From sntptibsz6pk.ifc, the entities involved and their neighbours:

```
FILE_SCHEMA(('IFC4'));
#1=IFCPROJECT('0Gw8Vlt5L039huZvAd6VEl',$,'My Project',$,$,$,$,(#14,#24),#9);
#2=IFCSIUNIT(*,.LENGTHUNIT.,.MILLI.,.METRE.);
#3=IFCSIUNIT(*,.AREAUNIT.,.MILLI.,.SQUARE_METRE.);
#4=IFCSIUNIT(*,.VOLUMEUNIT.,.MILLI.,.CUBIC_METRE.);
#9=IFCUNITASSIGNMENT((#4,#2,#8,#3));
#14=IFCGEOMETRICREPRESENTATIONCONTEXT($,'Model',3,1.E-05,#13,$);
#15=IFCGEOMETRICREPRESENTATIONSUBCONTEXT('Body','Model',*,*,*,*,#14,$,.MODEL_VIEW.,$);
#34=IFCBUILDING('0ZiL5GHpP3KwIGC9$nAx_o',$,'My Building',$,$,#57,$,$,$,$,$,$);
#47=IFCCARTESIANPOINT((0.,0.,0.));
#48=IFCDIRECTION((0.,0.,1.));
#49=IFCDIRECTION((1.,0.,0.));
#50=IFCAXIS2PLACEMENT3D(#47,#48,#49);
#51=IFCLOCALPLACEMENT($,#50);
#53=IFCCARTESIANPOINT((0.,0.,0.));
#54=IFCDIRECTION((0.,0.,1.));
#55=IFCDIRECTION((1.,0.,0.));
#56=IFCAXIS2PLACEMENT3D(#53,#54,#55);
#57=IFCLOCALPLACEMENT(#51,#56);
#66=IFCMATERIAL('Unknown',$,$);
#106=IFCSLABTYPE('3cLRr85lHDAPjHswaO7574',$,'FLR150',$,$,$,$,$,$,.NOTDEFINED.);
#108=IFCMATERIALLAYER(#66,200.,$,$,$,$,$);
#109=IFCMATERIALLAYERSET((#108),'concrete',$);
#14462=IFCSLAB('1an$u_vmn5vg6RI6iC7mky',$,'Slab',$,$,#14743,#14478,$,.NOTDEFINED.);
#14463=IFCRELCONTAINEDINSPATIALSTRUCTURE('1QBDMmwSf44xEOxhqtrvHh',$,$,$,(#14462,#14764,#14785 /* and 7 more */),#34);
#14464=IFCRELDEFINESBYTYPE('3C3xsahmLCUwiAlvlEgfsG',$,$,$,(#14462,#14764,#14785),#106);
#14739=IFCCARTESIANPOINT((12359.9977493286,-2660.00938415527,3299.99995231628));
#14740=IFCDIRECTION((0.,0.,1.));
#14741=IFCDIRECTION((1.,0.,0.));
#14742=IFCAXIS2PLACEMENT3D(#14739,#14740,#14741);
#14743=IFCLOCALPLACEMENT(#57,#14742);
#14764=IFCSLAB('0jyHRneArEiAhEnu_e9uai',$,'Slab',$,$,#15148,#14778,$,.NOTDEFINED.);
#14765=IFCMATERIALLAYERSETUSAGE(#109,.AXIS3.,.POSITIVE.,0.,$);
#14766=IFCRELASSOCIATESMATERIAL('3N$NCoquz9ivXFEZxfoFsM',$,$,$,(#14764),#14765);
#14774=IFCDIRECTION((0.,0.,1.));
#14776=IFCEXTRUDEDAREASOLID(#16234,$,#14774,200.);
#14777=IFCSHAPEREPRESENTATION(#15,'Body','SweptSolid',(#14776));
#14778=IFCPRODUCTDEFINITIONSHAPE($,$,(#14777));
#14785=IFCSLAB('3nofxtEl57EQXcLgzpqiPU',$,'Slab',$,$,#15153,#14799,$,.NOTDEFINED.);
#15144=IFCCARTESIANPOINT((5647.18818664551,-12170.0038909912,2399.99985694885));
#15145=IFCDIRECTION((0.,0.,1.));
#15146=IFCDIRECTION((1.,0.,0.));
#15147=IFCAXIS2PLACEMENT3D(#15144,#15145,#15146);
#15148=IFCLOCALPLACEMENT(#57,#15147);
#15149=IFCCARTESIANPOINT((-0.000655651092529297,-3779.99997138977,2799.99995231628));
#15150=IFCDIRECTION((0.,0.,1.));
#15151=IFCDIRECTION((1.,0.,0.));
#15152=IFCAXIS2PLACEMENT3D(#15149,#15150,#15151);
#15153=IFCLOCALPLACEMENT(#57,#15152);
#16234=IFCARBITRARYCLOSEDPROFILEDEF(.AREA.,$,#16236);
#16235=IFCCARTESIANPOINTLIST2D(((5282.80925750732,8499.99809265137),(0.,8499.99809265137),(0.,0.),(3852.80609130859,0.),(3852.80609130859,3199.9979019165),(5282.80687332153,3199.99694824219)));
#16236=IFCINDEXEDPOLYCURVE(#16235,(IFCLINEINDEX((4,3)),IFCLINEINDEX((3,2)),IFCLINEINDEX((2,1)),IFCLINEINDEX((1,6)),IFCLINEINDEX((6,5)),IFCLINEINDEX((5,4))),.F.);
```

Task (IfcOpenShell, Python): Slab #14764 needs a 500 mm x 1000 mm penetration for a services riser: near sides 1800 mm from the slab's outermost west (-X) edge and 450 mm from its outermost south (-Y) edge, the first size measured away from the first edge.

```python
import numpy as np
import ifcopenshell
import ifcopenshell.api.feature
import ifcopenshell.api.geometry
import ifcopenshell.api.root
import ifcopenshell.geom
import ifcopenshell.util.placement
import ifcopenshell.util.representation
import ifcopenshell.util.shape
import ifcopenshell.util.unit

model = ifcopenshell.open("sntptibsz6pk.ifc")
unit_scale = ifcopenshell.util.unit.calculate_unit_scale(model)
settings = ifcopenshell.geom.settings()


def volume(element):
    """Net volume in cubic metres, openings subtracted."""
    shape = ifcopenshell.geom.create_shape(settings, element)
    return ifcopenshell.util.shape.get_volume(shape.geometry)


slab = model.by_guid("0jyHRneArEiAhEnu_e9uai")
before = volume(slab)

# Extent in the slab's own axes, in metres. The edges named are its -X and -Y sides.
slab_shape = ifcopenshell.geom.create_shape(settings, slab)
vertices = ifcopenshell.util.shape.get_vertices(slab_shape.geometry)
x_min, y_min, bottom = vertices.min(axis=0)
top = vertices[:, 2].max()

opening = ifcopenshell.api.root.create_entity(model, ifc_class="IfcOpeningElement", name="Services riser opening", predefined_type="OPENING")
context = ifcopenshell.util.representation.get_context(model, "Model", "Body", "MODEL_VIEW")
width, depth = 0.5, 1
outline = [(0.0, 0.0), (width, 0.0), (width, depth), (0.0, depth), (0.0, 0.0)]
# Overshoot both faces by 50 mm so the cut is clean.
shape = ifcopenshell.api.geometry.add_slab_representation(
    model, context=context, depth=top - bottom + 0.1, polyline=outline
)
ifcopenshell.api.geometry.assign_representation(model, product=opening, representation=shape)

matrix = ifcopenshell.util.placement.get_local_placement(slab.ObjectPlacement)
matrix[:, 3] = matrix @ np.append(np.array([x_min + 1.8, y_min + 0.45, bottom - 0.05]) / unit_scale, 1.0)
ifcopenshell.api.geometry.edit_object_placement(model, product=opening, matrix=matrix, is_si=False)
ifcopenshell.api.feature.add_feature(model, feature=opening, element=slab)

after = volume(slab)

print(f"slab volume {before:.3f} -> {after:.3f} m3")

model.write("sntptibsz6pk_updated.ifc")
```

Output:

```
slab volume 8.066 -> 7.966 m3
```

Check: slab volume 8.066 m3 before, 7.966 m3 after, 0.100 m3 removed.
